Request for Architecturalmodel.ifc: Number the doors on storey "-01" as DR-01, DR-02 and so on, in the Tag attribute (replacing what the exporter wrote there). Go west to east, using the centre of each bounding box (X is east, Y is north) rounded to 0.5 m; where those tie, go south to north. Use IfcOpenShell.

First a look at what the model holds.

```python
import ifcopenshell
import ifcopenshell.util.element
import ifcopenshell.util.placement

model = ifcopenshell.open("Architecturalmodel.ifc")
print(model.schema)
storey = next(s for s in model.by_type("IfcBuildingStorey") if s.Name == "-01")
doors = [e for e in ifcopenshell.util.element.get_decomposition(storey) if e.is_a("IfcDoor")]
for e in sorted(doors, key=lambda e: e.id()):
    origin = ifcopenshell.util.placement.get_local_placement(e.ObjectPlacement)[:3, 3]
    print(e.id(), e.Tag, e.Name, origin.round(2) + 0.0, sep=" | ")
```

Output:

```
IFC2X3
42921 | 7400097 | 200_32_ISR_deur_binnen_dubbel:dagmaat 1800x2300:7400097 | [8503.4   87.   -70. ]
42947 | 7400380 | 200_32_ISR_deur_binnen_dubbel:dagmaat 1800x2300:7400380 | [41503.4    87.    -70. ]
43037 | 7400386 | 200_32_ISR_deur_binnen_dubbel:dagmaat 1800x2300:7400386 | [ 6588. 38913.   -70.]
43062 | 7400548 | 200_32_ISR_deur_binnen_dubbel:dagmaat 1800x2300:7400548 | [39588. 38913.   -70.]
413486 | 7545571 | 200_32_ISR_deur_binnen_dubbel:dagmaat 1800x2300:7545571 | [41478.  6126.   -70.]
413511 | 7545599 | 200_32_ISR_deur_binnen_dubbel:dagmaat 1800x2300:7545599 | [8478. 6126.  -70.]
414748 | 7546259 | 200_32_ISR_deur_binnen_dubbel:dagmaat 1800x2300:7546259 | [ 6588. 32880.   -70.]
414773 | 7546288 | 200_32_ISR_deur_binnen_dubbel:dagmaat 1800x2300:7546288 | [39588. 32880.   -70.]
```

```python
import ifcopenshell
import ifcopenshell.geom
import ifcopenshell.util.element
import ifcopenshell.util.shape

model = ifcopenshell.open("Architecturalmodel.ifc")
settings = ifcopenshell.geom.settings()
settings.set("use-world-coords", True)


def centre(element):
    shape = ifcopenshell.geom.create_shape(settings, element)
    return ifcopenshell.util.shape.get_bbox_centroid(shape.geometry)


storey = next(s for s in model.by_type("IfcBuildingStorey") if s.Name == "-01")
doors = [e for e in ifcopenshell.util.element.get_decomposition(storey) if e.is_a("IfcDoor")]

# Insertion points can sit at a corner or the storey origin, so sort by the geometry (in metres).
centres = {e: centre(e) for e in doors}
doors.sort(key=lambda e: (round(centres[e][0] / 0.5), centres[e][1]))

for i, e in enumerate(doors, start=1):
    number = f"DR-{i:02d}"
    e.Tag = number
    print(e.id(), number)

model.write("Architecturalmodel_rev.ifc")
```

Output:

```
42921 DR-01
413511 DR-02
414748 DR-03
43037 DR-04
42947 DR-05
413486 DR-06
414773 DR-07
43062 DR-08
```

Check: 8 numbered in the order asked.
